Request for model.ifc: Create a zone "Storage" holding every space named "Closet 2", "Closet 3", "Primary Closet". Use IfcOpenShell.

First a look at what the model holds.

```python
import ifcopenshell

model = ifcopenshell.open("model.ifc")
print(model.schema)
seen = {}
for space in model.by_type("IfcSpace"):
    seen[space.LongName] = seen.get(space.LongName, 0) + 1
for name, count in sorted(seen.items(), key=str):
    print(count, "x", name)
print("zones:", [z.Name for z in model.by_type("IfcZone")][:20])
```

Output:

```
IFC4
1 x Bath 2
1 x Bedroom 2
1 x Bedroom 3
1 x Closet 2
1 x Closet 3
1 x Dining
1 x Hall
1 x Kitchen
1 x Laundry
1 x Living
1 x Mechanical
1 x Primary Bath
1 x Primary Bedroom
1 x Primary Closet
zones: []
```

```python
import ifcopenshell
import ifcopenshell.api.group
import ifcopenshell.api.root

model = ifcopenshell.open("model.ifc")

names = {"Closet 2", "Closet 3", "Primary Closet"}
spaces = [s for s in model.by_type("IfcSpace") if s.LongName in names]

zone = ifcopenshell.api.root.create_entity(model, ifc_class="IfcZone", name="Storage")
ifcopenshell.api.group.assign_group(model, products=spaces, group=zone)
print(len(spaces), "spaces in", zone.Name)

model.write("model_v2.ifc")
```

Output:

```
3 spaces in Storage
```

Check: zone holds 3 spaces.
